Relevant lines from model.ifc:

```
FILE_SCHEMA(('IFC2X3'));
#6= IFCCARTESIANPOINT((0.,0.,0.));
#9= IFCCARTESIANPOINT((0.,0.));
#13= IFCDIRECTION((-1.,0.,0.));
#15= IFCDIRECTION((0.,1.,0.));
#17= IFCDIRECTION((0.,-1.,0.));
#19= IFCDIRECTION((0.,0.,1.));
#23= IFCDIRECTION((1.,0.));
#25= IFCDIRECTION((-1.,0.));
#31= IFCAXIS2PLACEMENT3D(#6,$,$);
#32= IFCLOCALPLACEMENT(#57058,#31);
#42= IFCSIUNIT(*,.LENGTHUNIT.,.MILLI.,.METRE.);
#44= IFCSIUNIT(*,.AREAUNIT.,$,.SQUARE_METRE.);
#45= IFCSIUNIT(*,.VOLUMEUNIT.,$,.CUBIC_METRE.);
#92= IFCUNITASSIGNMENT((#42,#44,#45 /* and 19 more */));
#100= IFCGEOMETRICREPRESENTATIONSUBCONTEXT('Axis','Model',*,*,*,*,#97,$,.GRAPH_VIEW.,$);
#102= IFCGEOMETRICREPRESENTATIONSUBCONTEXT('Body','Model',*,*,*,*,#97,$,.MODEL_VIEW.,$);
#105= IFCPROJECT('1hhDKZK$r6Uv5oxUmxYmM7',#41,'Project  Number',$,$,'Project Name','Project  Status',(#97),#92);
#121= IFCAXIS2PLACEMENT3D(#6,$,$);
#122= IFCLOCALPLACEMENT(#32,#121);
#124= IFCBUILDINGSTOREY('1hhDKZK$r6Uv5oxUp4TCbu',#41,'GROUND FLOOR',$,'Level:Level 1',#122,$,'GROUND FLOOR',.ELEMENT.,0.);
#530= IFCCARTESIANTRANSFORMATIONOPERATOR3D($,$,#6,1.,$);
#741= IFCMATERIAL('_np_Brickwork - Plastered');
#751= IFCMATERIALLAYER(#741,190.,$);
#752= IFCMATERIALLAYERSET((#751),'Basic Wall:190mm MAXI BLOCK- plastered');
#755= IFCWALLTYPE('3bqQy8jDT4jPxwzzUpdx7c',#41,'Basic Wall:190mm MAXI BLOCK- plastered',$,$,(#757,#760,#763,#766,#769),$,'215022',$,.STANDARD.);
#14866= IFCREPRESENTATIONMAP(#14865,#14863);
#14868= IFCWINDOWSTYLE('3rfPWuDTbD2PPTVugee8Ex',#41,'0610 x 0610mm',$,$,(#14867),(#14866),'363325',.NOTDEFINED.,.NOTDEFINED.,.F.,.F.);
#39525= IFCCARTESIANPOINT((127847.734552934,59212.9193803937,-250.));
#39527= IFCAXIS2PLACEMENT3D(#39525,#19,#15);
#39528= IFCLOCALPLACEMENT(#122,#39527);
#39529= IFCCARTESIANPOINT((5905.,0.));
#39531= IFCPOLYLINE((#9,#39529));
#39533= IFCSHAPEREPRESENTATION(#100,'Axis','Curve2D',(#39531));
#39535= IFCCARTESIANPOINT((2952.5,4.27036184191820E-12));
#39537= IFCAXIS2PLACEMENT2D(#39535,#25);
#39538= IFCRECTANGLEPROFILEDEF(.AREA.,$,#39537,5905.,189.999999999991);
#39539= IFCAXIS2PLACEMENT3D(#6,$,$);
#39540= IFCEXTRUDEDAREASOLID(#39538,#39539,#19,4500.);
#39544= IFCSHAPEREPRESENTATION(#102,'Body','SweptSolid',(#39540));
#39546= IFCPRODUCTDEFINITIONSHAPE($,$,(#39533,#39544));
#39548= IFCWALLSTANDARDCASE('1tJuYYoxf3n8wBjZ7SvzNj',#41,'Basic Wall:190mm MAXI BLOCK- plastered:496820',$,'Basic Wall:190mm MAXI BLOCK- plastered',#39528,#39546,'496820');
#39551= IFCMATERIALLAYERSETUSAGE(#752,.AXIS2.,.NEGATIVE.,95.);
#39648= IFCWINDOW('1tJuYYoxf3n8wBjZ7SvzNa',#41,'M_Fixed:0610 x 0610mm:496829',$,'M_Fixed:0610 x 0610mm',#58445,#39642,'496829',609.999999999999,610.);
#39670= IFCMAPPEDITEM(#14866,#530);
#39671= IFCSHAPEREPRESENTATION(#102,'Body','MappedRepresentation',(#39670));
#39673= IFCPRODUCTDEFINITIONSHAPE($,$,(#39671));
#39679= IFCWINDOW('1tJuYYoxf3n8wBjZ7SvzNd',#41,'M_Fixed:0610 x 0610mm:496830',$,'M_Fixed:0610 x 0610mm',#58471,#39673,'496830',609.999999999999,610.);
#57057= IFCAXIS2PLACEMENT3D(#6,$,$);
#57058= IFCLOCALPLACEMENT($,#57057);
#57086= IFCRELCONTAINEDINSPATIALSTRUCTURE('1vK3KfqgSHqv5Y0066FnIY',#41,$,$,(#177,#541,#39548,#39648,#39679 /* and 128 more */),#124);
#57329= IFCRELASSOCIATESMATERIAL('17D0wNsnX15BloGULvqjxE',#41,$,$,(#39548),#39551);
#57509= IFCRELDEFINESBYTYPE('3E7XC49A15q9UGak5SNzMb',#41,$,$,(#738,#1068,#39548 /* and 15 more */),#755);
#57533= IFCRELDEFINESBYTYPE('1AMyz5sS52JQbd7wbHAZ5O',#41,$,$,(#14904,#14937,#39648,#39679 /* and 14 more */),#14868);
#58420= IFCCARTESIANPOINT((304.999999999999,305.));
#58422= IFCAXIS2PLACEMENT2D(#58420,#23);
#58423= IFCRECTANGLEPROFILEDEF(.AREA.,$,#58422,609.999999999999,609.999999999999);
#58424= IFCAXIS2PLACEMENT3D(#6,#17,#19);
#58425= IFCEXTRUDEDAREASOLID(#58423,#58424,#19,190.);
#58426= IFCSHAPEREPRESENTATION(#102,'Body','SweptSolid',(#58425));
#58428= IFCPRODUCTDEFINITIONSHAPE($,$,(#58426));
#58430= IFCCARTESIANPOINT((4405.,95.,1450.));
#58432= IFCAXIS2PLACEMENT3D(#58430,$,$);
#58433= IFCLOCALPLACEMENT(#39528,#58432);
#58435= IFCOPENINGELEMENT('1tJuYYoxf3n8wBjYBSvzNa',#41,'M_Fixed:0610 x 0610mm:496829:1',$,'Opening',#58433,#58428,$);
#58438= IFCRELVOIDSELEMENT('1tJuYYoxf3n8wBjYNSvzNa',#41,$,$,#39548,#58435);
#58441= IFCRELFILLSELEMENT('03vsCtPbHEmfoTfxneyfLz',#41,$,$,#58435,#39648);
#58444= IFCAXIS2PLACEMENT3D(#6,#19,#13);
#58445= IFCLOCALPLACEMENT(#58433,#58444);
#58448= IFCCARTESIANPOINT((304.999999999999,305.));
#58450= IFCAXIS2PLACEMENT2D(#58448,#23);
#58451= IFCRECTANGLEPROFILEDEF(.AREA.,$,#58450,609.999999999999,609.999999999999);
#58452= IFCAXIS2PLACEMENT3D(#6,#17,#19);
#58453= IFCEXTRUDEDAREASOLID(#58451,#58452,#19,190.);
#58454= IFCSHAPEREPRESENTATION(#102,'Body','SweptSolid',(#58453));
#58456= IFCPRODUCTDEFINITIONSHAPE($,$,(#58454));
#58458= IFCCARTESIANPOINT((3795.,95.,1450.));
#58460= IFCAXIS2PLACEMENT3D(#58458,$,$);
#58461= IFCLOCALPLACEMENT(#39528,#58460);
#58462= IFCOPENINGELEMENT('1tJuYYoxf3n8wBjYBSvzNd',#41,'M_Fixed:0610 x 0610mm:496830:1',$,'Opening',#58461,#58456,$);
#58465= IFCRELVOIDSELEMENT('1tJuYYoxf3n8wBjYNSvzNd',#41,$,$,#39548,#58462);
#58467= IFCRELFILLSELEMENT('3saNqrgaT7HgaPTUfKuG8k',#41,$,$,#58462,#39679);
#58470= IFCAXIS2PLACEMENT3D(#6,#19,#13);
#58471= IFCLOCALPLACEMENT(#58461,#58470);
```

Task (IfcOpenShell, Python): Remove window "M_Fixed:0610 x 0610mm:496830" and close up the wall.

```python
import ifcopenshell
import ifcopenshell.api.feature
import ifcopenshell.api.root
import ifcopenshell.geom
import ifcopenshell.util.shape

model = ifcopenshell.open("model.ifc")
settings = ifcopenshell.geom.settings()


def volume(element):
    """Net volume in cubic metres, openings subtracted."""
    shape = ifcopenshell.geom.create_shape(settings, element)
    return ifcopenshell.util.shape.get_volume(shape.geometry)


window = model.by_guid("1tJuYYoxf3n8wBjZ7SvzNd")
opening = window.FillsVoids[0].RelatingOpeningElement
wall = opening.VoidsElements[0].RelatingBuildingElement
before = volume(wall)

ifcopenshell.api.root.remove_product(model, product=window)
ifcopenshell.api.feature.remove_feature(model, feature=opening)

after = volume(wall)

print(f"wall volume {before:.3f} -> {after:.3f} m3")

model.write("model_edited.ifc")
```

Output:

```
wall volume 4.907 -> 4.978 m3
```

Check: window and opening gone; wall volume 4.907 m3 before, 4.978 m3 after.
